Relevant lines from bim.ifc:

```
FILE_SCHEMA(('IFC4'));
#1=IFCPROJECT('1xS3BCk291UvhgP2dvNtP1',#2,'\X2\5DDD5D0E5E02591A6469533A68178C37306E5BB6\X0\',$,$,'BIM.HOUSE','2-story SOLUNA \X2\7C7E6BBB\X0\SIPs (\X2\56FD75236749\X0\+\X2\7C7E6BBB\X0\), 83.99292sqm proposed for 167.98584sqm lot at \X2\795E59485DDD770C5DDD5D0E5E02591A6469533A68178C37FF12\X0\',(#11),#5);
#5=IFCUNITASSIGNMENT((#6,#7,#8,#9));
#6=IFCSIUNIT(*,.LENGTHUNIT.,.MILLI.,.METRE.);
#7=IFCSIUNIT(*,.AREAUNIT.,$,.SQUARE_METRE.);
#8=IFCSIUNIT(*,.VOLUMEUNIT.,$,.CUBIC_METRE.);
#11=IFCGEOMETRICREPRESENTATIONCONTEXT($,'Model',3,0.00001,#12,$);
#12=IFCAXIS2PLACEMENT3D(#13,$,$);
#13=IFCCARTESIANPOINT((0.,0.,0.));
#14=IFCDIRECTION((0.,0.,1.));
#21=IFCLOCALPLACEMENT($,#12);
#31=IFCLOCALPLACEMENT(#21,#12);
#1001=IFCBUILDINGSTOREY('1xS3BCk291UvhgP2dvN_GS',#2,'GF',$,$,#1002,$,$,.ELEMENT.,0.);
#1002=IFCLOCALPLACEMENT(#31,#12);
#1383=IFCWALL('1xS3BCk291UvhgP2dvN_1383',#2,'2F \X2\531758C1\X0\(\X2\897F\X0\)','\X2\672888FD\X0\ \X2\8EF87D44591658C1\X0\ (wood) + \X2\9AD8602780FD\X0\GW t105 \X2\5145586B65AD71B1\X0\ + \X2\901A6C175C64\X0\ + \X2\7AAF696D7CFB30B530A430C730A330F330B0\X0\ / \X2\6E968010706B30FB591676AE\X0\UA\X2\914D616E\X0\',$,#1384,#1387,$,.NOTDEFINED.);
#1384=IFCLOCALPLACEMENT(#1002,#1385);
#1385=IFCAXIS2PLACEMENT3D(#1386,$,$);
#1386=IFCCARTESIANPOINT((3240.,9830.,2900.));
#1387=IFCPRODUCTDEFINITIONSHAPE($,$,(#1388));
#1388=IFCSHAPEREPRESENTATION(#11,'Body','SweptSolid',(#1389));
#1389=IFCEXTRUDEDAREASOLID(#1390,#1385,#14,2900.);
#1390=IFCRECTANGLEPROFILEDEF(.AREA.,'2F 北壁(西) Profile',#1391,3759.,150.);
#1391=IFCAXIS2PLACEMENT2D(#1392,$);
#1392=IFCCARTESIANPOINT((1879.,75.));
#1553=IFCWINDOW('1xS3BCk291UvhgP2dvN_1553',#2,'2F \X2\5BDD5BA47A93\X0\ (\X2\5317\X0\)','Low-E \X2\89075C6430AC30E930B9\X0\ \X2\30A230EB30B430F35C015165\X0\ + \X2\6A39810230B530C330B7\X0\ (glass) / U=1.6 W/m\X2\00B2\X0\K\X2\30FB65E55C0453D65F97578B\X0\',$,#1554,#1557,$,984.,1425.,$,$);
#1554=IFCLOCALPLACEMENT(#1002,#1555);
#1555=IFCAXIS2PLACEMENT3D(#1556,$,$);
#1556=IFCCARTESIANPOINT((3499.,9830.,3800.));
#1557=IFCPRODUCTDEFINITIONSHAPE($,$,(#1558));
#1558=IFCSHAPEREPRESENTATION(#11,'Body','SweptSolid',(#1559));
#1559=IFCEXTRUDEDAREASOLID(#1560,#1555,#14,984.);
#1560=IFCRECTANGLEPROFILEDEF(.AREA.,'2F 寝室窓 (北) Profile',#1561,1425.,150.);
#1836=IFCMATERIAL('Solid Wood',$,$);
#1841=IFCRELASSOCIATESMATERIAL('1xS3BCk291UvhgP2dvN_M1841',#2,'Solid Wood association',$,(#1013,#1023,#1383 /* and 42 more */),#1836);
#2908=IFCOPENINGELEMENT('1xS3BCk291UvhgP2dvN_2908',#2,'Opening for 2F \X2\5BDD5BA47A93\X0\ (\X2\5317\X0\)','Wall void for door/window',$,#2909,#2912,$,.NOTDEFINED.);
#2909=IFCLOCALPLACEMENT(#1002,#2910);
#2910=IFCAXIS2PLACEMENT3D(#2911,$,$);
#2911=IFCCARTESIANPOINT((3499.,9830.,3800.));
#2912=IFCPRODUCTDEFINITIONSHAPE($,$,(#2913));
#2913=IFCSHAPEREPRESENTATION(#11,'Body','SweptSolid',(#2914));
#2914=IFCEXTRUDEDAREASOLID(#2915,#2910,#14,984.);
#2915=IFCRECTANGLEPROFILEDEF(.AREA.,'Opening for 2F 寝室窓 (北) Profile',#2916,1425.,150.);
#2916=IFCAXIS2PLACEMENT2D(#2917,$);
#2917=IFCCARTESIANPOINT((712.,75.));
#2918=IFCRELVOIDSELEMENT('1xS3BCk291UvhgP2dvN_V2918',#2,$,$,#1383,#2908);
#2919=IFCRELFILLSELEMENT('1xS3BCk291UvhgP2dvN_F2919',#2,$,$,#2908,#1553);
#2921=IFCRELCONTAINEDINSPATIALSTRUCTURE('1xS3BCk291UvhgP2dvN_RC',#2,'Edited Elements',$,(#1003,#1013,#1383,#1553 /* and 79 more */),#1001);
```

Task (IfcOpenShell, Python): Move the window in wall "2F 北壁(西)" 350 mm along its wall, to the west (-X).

```python
import ifcopenshell
import ifcopenshell.api.geometry
import ifcopenshell.util.placement

model = ifcopenshell.open("bim.ifc")

window = model.by_guid("1xS3BCk291UvhgP2dvN_1553")
opening = window.FillsVoids[0].RelatingOpeningElement
wall = opening.VoidsElements[0].RelatingBuildingElement

wall_matrix = ifcopenshell.util.placement.get_local_placement(wall.ObjectPlacement)
shift = wall_matrix[:3, 0] * -350.0
before = ifcopenshell.util.placement.get_local_placement(window.ObjectPlacement)[:3, 3].copy()

# The window is not placed relative to its opening, so move both.
for product in (opening, window):
    matrix = ifcopenshell.util.placement.get_local_placement(product.ObjectPlacement)
    matrix[:3, 3] += shift
    ifcopenshell.api.geometry.edit_object_placement(model, product=product, matrix=matrix, is_si=False)

after = ifcopenshell.util.placement.get_local_placement(window.ObjectPlacement)[:3, 3]
print("window moved by", (after - before).round(3) + 0.0)

model.write("bim_rev.ifc")
```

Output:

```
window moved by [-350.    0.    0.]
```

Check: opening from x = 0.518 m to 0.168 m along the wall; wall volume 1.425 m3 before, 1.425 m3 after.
